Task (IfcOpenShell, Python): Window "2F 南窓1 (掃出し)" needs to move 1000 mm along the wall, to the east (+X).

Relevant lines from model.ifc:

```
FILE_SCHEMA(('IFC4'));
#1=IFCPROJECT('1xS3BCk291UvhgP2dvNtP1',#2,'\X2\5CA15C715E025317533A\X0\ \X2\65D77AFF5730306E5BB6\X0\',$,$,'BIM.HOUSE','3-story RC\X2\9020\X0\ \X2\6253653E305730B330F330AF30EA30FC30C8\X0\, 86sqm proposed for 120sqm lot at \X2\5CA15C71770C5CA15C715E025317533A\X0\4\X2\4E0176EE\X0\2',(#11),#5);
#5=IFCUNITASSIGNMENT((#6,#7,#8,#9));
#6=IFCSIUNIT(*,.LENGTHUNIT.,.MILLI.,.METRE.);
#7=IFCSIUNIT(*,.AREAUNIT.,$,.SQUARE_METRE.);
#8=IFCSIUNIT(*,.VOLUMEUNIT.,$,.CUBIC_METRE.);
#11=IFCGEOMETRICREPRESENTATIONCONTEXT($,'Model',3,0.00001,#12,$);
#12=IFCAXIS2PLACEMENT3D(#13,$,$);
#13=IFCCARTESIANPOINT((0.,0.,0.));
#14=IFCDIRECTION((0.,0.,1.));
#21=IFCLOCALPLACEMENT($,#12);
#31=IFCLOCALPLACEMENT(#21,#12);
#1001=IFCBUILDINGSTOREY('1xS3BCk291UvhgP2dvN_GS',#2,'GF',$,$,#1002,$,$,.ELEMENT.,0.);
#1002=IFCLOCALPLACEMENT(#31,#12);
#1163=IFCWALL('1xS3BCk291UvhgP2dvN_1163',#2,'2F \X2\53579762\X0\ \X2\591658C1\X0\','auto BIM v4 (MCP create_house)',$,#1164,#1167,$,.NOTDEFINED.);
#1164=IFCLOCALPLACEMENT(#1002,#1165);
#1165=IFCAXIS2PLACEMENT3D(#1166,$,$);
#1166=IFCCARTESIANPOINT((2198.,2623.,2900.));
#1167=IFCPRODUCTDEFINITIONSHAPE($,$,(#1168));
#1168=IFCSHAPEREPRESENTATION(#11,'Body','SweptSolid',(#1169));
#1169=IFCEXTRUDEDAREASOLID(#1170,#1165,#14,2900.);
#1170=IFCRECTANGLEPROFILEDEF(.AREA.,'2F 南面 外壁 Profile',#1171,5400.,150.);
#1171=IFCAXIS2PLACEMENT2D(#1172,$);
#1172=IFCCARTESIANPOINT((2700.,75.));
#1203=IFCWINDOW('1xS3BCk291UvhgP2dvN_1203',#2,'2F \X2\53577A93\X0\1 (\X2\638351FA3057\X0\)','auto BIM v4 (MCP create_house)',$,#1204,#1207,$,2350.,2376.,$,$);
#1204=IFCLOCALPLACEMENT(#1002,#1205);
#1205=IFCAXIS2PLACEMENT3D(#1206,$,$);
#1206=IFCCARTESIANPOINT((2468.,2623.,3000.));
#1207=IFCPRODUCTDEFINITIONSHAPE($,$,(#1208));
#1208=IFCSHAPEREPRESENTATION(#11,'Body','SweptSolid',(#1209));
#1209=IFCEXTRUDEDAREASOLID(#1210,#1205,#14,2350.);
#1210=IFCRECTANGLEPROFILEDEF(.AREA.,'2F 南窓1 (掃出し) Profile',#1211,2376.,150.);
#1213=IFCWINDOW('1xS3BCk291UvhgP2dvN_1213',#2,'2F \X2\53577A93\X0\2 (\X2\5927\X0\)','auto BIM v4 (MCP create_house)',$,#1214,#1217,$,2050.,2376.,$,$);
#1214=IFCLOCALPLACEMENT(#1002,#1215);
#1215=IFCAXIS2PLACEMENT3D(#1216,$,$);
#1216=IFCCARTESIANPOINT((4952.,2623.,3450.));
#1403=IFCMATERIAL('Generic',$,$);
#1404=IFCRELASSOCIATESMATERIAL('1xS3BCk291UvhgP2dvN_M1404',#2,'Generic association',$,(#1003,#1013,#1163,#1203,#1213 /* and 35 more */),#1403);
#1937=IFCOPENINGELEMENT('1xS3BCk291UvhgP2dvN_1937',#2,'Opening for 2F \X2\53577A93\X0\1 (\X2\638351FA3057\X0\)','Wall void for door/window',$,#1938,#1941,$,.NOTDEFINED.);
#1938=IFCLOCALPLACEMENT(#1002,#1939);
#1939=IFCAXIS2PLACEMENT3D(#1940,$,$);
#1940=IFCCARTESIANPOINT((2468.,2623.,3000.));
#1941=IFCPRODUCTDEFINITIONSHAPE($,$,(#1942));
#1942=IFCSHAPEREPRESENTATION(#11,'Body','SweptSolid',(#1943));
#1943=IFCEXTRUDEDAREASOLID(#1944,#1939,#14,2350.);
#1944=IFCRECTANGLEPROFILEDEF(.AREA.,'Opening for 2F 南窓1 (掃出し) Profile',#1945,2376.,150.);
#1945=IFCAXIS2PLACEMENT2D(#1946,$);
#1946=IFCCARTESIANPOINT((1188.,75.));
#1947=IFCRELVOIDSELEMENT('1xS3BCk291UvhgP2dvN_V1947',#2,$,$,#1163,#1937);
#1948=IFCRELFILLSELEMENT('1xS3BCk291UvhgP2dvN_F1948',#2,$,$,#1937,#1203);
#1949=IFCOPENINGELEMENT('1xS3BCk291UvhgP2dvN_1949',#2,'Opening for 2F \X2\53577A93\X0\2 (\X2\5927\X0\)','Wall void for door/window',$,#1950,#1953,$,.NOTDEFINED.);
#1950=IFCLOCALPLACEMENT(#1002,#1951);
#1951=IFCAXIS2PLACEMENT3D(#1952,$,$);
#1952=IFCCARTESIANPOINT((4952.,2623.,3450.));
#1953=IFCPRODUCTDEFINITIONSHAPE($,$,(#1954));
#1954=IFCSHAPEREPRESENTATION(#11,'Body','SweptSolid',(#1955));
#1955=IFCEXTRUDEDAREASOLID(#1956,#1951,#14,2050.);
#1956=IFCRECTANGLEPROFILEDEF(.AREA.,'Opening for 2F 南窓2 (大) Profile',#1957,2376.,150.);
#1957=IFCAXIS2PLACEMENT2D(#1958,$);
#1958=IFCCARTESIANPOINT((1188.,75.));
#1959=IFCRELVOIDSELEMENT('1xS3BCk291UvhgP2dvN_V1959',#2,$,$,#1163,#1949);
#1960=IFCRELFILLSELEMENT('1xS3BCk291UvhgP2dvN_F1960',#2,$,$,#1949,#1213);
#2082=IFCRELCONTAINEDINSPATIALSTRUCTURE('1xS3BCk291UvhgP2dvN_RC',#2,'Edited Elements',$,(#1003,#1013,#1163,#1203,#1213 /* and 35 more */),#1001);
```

```python
import ifcopenshell
import ifcopenshell.api.geometry
import ifcopenshell.util.placement
import ifcopenshell.util.unit

model = ifcopenshell.open("model.ifc")
unit_scale = ifcopenshell.util.unit.calculate_unit_scale(model)

window = model.by_guid("1xS3BCk291UvhgP2dvN_1203")
opening = window.FillsVoids[0].RelatingOpeningElement
wall = opening.VoidsElements[0].RelatingBuildingElement

wall_matrix = ifcopenshell.util.placement.get_local_placement(wall.ObjectPlacement)
shift = wall_matrix[:3, 0] * 1 / unit_scale
before = ifcopenshell.util.placement.get_local_placement(window.ObjectPlacement)[:3, 3].copy()

# The window is not placed relative to its opening, so move both.
for product in (opening, window):
    matrix = ifcopenshell.util.placement.get_local_placement(product.ObjectPlacement)
    matrix[:3, 3] += shift
    ifcopenshell.api.geometry.edit_object_placement(model, product=product, matrix=matrix, is_si=False)

after = ifcopenshell.util.placement.get_local_placement(window.ObjectPlacement)[:3, 3]
print("window moved by", (after - before).round(3) + 0.0)

model.write("model-out.ifc")
```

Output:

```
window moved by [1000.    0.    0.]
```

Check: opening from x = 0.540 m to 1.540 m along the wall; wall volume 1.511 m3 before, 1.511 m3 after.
